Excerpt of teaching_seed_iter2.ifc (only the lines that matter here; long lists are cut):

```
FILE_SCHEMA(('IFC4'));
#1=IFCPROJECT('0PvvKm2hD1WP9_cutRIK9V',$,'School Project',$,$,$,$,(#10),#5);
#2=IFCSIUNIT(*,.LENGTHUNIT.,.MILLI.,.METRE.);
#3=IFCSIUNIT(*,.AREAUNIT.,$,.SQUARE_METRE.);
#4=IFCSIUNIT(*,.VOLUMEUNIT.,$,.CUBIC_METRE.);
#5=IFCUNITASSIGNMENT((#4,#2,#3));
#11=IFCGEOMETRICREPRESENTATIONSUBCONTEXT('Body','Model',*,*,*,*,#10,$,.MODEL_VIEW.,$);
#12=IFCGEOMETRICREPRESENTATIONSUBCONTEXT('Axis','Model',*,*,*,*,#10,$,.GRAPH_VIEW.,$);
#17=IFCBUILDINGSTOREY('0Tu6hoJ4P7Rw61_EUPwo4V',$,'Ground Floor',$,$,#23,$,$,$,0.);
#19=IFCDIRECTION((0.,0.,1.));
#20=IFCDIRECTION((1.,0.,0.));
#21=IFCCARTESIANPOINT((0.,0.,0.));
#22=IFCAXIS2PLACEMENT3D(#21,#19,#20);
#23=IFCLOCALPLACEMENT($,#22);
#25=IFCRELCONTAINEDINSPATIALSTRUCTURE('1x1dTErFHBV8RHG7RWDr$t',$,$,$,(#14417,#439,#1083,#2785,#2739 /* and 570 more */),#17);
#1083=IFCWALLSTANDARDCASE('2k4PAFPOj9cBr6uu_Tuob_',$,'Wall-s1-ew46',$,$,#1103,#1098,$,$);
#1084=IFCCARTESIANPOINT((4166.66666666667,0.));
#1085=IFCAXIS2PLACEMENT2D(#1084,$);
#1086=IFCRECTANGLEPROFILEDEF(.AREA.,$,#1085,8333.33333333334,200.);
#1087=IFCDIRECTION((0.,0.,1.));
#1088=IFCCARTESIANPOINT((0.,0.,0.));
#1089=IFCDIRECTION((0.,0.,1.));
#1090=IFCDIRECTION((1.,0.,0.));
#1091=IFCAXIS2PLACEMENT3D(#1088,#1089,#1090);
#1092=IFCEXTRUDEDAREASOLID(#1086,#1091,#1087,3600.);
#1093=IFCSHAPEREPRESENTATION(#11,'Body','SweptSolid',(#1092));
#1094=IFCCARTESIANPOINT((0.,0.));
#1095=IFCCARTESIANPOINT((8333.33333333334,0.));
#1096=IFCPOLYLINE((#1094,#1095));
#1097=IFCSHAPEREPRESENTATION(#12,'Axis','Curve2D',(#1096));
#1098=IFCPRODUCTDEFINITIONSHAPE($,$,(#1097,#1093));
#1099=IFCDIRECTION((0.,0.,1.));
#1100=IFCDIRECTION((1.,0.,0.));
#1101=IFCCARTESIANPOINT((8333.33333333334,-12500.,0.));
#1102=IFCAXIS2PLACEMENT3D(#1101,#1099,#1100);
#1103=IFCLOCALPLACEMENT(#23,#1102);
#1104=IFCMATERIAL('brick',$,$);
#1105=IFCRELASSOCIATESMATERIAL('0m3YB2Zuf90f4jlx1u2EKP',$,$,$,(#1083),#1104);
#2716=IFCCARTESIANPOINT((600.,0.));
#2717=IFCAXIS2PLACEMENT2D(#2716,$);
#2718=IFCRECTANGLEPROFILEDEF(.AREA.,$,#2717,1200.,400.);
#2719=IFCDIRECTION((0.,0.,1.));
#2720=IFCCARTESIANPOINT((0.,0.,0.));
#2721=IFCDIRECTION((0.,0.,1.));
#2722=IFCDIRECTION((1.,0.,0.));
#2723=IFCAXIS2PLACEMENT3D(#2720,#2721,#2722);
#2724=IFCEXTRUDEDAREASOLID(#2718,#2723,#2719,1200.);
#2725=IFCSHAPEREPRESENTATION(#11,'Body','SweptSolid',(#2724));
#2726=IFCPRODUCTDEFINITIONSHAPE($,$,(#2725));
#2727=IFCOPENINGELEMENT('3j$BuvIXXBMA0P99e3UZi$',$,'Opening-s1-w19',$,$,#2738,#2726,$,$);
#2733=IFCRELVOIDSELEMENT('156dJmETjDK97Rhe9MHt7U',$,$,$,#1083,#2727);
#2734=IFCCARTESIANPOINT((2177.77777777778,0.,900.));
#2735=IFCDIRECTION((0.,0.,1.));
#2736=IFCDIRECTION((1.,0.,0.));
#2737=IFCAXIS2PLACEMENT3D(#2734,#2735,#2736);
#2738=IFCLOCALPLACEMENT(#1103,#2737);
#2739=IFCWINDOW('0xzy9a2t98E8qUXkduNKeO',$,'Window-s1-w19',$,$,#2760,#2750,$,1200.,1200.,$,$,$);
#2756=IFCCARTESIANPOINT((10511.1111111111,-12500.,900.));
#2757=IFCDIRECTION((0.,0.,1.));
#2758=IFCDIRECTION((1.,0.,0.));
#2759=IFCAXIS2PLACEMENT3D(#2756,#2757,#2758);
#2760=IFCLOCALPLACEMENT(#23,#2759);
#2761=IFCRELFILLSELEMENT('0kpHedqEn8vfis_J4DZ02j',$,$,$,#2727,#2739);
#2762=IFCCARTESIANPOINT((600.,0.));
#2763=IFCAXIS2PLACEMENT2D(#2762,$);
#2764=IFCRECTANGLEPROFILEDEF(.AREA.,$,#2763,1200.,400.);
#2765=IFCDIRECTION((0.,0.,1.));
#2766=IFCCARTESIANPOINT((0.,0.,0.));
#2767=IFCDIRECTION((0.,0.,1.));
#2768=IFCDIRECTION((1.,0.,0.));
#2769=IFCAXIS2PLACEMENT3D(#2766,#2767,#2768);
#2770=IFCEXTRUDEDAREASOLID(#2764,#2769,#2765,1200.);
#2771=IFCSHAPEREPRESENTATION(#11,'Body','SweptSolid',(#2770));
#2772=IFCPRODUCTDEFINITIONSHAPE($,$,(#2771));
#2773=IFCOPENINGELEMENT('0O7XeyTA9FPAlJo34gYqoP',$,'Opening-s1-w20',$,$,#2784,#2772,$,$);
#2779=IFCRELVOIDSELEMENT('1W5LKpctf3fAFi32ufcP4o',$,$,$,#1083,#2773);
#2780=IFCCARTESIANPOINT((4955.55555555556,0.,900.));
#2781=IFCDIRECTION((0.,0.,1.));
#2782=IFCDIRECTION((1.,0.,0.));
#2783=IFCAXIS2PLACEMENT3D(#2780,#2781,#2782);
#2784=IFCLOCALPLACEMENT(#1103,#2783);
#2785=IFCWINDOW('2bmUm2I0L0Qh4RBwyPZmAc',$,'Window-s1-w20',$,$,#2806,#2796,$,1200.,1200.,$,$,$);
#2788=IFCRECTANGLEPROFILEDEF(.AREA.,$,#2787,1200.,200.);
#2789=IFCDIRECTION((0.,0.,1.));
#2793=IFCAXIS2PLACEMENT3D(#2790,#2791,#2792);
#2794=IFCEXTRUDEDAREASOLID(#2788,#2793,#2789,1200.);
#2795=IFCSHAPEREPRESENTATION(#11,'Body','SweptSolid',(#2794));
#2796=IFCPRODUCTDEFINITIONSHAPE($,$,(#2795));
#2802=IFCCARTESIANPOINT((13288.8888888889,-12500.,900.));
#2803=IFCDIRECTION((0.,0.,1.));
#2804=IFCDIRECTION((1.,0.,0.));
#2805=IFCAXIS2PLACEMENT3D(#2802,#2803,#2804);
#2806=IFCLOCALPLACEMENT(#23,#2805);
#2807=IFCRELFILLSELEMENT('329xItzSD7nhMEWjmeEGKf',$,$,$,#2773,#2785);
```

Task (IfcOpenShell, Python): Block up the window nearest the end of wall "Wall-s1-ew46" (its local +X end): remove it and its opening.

```python
import ifcopenshell
import ifcopenshell.api.feature
import ifcopenshell.api.root
import ifcopenshell.geom
import ifcopenshell.util.shape

model = ifcopenshell.open("teaching_seed_iter2.ifc")
settings = ifcopenshell.geom.settings()


def volume(element):
    """Net volume in cubic metres, openings subtracted."""
    shape = ifcopenshell.geom.create_shape(settings, element)
    return ifcopenshell.util.shape.get_volume(shape.geometry)


window = model.by_id(2785)
opening = window.FillsVoids[0].RelatingOpeningElement
wall = opening.VoidsElements[0].RelatingBuildingElement
before = volume(wall)

ifcopenshell.api.root.remove_product(model, product=window)
ifcopenshell.api.feature.remove_feature(model, feature=opening)

after = volume(wall)

print(f"wall volume {before:.3f} -> {after:.3f} m3")

model.write("teaching_seed_iter2_edited.ifc")
```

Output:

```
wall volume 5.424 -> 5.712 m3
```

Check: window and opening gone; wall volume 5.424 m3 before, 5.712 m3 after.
